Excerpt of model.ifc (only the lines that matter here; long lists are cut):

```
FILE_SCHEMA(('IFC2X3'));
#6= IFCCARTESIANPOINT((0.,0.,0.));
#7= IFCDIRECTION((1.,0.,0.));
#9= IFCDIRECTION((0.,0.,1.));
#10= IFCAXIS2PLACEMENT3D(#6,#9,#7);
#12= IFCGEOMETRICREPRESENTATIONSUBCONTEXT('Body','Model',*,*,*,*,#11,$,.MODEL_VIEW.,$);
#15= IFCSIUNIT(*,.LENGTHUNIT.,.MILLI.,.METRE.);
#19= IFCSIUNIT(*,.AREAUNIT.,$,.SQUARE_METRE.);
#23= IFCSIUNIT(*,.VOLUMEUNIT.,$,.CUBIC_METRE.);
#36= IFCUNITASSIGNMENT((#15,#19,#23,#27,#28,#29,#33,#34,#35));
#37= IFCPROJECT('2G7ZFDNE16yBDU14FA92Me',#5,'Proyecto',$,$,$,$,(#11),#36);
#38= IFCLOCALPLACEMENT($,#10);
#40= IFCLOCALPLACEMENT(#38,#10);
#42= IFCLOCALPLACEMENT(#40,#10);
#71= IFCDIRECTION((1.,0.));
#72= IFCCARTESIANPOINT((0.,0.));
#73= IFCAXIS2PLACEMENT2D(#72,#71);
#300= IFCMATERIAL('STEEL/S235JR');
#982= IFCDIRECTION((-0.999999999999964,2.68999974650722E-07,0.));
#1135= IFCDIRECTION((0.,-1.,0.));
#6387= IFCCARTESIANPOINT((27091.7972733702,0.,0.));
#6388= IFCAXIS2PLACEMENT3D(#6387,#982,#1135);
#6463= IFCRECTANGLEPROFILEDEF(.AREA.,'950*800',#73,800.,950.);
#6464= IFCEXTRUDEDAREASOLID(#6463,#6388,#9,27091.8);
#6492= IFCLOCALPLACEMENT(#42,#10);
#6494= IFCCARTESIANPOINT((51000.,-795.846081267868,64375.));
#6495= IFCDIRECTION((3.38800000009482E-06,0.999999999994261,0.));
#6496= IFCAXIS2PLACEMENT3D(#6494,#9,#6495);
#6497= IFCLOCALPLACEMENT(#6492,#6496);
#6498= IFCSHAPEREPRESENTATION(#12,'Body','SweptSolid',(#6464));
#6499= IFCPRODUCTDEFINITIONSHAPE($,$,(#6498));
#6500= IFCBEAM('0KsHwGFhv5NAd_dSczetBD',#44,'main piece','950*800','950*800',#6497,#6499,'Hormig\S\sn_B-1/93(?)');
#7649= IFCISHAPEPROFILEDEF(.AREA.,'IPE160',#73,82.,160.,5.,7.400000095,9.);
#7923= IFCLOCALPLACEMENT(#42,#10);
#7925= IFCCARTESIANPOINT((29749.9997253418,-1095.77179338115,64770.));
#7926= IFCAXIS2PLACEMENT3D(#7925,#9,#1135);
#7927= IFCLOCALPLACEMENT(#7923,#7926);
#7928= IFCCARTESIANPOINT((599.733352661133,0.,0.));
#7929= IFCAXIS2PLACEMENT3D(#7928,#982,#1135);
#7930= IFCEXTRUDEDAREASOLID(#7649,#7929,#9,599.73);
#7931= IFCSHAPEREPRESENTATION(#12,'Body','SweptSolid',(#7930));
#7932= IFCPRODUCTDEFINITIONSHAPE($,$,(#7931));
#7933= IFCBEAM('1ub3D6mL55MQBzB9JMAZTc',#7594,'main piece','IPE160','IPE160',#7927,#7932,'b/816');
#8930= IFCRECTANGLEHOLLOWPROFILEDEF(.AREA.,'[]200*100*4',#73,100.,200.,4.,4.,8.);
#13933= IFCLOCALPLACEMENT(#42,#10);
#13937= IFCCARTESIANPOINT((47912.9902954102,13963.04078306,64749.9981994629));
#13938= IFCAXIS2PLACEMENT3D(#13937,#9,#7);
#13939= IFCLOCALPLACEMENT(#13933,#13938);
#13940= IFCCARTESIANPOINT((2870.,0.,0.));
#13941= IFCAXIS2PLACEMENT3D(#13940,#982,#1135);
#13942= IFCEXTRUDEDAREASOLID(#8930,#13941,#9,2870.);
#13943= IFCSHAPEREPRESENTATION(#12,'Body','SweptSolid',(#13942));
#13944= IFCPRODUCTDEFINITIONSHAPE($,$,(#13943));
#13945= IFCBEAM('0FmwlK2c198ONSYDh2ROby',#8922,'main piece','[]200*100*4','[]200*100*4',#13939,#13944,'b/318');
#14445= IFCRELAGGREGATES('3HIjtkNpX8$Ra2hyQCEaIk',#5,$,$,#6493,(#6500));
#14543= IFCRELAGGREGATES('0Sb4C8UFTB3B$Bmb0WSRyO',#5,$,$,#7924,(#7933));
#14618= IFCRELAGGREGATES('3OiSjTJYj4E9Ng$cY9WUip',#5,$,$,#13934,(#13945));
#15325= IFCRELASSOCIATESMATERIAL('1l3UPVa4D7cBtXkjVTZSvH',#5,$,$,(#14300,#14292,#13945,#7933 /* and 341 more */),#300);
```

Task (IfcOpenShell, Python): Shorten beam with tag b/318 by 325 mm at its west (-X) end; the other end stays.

```python
import ifcopenshell
import ifcopenshell.util.representation
import ifcopenshell.util.unit

model = ifcopenshell.open("model.ifc")
unit_scale = ifcopenshell.util.unit.calculate_unit_scale(model)

member = model.by_guid("0FmwlK2c198ONSYDh2ROby")
change = -0.325 / unit_scale

# The extrusion runs towards the end named, so only its depth changes.
body = ifcopenshell.util.representation.get_representation(member, "Model", "Body")
solid = body.Items[0]
old_length = solid.Depth
solid.Depth += change

print(f"length {old_length:g} -> {solid.Depth:g}")

model.write("model_updated.ifc")
```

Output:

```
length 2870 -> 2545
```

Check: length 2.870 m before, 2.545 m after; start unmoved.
